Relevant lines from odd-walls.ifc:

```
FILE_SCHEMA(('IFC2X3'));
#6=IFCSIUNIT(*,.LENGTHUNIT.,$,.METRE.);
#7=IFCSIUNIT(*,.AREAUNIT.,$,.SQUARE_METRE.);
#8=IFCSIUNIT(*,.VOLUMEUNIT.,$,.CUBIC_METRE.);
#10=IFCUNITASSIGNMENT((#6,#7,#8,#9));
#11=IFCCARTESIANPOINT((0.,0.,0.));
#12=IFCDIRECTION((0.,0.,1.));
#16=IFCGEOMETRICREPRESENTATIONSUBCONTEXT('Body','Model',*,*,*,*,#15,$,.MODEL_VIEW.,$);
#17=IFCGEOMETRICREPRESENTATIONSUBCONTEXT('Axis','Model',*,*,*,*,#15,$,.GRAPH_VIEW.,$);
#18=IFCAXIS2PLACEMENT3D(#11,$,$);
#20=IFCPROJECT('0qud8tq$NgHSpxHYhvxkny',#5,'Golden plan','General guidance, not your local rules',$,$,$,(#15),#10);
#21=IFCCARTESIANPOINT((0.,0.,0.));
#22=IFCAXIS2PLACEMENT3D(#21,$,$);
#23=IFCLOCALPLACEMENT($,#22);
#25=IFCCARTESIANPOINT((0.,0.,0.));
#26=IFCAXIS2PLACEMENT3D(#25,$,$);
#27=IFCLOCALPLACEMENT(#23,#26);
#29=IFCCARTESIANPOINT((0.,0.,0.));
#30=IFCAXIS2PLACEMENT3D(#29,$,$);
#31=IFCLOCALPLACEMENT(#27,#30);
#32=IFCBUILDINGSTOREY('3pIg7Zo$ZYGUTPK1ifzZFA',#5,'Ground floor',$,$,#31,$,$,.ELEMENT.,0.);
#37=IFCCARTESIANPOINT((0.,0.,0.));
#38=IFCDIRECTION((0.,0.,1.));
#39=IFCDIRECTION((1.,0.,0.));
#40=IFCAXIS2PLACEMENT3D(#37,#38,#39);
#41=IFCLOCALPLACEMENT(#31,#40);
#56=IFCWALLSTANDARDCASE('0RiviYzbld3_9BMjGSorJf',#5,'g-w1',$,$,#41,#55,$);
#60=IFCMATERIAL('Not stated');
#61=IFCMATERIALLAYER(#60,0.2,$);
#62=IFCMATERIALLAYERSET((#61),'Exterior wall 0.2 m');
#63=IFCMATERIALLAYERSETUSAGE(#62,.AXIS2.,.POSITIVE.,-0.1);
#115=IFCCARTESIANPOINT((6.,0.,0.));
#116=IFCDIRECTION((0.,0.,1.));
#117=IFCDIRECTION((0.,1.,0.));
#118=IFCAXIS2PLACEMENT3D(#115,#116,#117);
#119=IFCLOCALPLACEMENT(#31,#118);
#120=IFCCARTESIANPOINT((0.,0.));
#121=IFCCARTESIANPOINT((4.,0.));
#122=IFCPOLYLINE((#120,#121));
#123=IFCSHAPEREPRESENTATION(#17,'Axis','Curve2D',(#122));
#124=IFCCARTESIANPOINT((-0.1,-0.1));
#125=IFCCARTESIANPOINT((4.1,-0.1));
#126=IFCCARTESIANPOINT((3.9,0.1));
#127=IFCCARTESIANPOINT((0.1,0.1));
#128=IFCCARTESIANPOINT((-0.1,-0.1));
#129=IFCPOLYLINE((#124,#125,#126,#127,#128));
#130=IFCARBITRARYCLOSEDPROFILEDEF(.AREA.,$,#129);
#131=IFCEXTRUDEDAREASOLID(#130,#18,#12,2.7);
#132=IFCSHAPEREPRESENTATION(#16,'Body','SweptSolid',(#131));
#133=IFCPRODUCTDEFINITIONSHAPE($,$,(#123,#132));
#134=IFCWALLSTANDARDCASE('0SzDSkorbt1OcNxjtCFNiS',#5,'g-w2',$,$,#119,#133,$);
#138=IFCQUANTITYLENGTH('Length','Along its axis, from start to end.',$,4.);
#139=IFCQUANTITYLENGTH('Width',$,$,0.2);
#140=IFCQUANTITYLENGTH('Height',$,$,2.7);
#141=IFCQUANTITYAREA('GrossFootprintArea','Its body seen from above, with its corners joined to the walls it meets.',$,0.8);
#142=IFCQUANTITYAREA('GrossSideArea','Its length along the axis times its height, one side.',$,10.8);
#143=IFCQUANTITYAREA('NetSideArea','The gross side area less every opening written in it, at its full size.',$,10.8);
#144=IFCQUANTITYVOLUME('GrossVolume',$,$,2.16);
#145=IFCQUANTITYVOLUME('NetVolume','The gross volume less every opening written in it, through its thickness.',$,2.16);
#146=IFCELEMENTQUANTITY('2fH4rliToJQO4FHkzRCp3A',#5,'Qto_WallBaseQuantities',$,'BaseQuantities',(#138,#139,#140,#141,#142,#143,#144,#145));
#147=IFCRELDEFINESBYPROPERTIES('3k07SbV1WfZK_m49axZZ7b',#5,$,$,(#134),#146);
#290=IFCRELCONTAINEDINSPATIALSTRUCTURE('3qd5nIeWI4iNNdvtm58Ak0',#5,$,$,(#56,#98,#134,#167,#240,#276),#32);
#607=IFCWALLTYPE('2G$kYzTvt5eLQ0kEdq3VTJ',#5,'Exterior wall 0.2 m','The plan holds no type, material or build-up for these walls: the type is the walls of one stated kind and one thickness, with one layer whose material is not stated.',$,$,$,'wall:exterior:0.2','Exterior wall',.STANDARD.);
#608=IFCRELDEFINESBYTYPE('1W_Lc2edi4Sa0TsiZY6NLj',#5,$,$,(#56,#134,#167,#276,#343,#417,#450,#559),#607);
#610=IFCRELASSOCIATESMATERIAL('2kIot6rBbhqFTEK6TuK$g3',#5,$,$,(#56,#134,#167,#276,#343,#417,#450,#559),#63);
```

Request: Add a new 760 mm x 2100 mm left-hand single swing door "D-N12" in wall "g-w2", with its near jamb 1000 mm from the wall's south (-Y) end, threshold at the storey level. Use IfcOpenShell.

```python
import numpy as np
import ifcopenshell
import ifcopenshell.api.feature
import ifcopenshell.api.geometry
import ifcopenshell.api.pset
import ifcopenshell.api.root
import ifcopenshell.api.spatial
import ifcopenshell.api.type
import ifcopenshell.geom
import ifcopenshell.util.element
import ifcopenshell.util.placement
import ifcopenshell.util.representation
import ifcopenshell.util.shape
import ifcopenshell.util.unit

model = ifcopenshell.open("odd-walls.ifc")
unit_scale = ifcopenshell.util.unit.calculate_unit_scale(model)
area_scale = ifcopenshell.util.unit.calculate_unit_scale(model, "AREAUNIT")
volume_scale = ifcopenshell.util.unit.calculate_unit_scale(model, "VOLUMEUNIT")
settings = ifcopenshell.geom.settings()


def volume(element):
    """Net volume in cubic metres, openings subtracted."""
    shape = ifcopenshell.geom.create_shape(settings, element)
    return ifcopenshell.util.shape.get_volume(shape.geometry)


wall = model.by_guid("0SzDSkorbt1OcNxjtCFNiS")
storey = ifcopenshell.util.element.get_container(wall, ifc_class="IfcBuildingStorey")
context = ifcopenshell.util.representation.get_context(model, "Model", "Body", "MODEL_VIEW")
before = volume(wall)

width, height, from_end, sill = 0.76, 2.1, 1, 0.0  # metres

# The wall runs along its own X axis, and the end named is its -X end.
wall_shape = ifcopenshell.geom.create_shape(settings, wall)
x, y, z = ifcopenshell.util.shape.get_vertices(wall_shape.geometry).T
start = x.min() + from_end
face, thickness = float(y.min()), float(y.max() - y.min())
wall_matrix = ifcopenshell.util.placement.get_local_placement(wall.ObjectPlacement)
level = ifcopenshell.util.placement.get_local_placement(storey.ObjectPlacement)[2, 3]


def in_wall(x, y):
    """Placement at x, y metres in the wall's axes, at sill height."""
    matrix = wall_matrix.copy()
    matrix[:, 3] = wall_matrix @ np.array([x / unit_scale, y / unit_scale, 0.0, 1.0])
    matrix[2, 3] = level + sill / unit_scale
    return matrix


# Opening: a box that overshoots both wall faces by 50 mm.
opening = ifcopenshell.api.root.create_entity(model, ifc_class="IfcOpeningElement")
box = ifcopenshell.api.geometry.add_wall_representation(
    model, context=context, length=width, height=height, thickness=thickness + 0.1
)
ifcopenshell.api.geometry.assign_representation(model, product=opening, representation=box)
ifcopenshell.api.geometry.edit_object_placement(model, product=opening, matrix=in_wall(start, face - 0.05), is_si=False)
ifcopenshell.api.feature.add_feature(model, feature=opening, element=wall)

door = ifcopenshell.api.root.create_entity(model, ifc_class="IfcDoor", name="D-N12")
door.OverallWidth, door.OverallHeight = width / unit_scale, height / unit_scale
body = ifcopenshell.api.geometry.add_door_representation(
    model,
    context=context,
    overall_width=door.OverallWidth,
    overall_height=door.OverallHeight,
    operation_type="SINGLE_SWING_LEFT",
    lining_properties={"LiningDepth": thickness / unit_scale, "ThresholdDepth": thickness / unit_scale},
)
ifcopenshell.api.geometry.assign_representation(model, product=door, representation=body)
ifcopenshell.api.spatial.assign_container(model, products=[door], relating_structure=storey)
fills = ifcopenshell.api.feature.add_filling(model, opening=opening, element=door)
fills.OwnerHistory = door.OwnerHistory  # required in IFC2X3

# IFC2X3 keeps the operation on the door style.
style = ifcopenshell.api.root.create_entity(model, ifc_class="IfcDoorStyle", name="D-N12")
style.OperationType, style.ConstructionType = "SINGLE_SWING_LEFT", "NOTDEFINED"
style.ParameterTakesPrecedence = style.Sizeable = False
ifcopenshell.api.type.assign_type(model, related_objects=[door], relating_type=style)

# The lining spans the wall, so the door starts at the wall face.
ifcopenshell.api.geometry.edit_object_placement(model, product=door, matrix=in_wall(start, face), is_si=False)

after = volume(wall)

# Update the wall's stored quantities.
qto = model.by_id(ifcopenshell.util.element.get_pset(wall, "Qto_WallBaseQuantities", should_inherit=False)["id"])
ifcopenshell.api.pset.edit_qto(model, qto=qto, properties={
    "NetSideArea": after / thickness / area_scale,
    "NetVolume": after / volume_scale,
})

print(f"wall volume {before:.3f} -> {after:.3f} m3")

model.write("odd-walls_rev.ifc")
```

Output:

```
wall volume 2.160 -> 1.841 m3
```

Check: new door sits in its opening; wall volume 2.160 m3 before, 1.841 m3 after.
